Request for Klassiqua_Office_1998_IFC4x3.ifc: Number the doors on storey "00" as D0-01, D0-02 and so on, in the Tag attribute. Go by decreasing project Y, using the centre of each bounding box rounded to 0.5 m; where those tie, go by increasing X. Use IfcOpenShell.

First a look at what the model holds.

```python
import ifcopenshell
import ifcopenshell.util.element
import ifcopenshell.util.placement

model = ifcopenshell.open("Klassiqua_Office_1998_IFC4x3.ifc")
print(model.schema)
storey = next(s for s in model.by_type("IfcBuildingStorey") if s.Name == "00")
doors = [e for e in ifcopenshell.util.element.get_decomposition(storey) if e.is_a("IfcDoor")]
for e in sorted(doors, key=lambda e: e.id()):
    origin = ifcopenshell.util.placement.get_local_placement(e.ObjectPlacement)[:3, 3]
    print(e.id(), e.Tag, e.Name, origin.round(2) + 0.0, sep=" | ")
```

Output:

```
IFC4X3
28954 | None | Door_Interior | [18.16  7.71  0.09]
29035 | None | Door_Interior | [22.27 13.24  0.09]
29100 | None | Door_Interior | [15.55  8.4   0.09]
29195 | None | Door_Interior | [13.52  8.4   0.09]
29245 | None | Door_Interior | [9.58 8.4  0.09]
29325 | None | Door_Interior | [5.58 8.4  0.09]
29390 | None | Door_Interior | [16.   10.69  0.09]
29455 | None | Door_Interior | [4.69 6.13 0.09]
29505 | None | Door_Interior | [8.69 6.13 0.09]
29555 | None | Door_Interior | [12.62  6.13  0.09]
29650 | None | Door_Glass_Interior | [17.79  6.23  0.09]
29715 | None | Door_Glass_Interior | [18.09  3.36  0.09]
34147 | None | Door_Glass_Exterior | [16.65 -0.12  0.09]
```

```python
import ifcopenshell
import ifcopenshell.geom
import ifcopenshell.util.element
import ifcopenshell.util.shape

model = ifcopenshell.open("Klassiqua_Office_1998_IFC4x3.ifc")
settings = ifcopenshell.geom.settings()
settings.set("use-world-coords", True)


def centre(element):
    shape = ifcopenshell.geom.create_shape(settings, element)
    return ifcopenshell.util.shape.get_bbox_centroid(shape.geometry)


storey = next(s for s in model.by_type("IfcBuildingStorey") if s.Name == "00")
doors = [e for e in ifcopenshell.util.element.get_decomposition(storey) if e.is_a("IfcDoor")]

# Insertion points can sit at a corner or the storey origin, so sort by the geometry (in metres).
centres = {e: centre(e) for e in doors}
doors.sort(key=lambda e: (-round(centres[e][1] / 0.5), centres[e][0]))

for i, e in enumerate(doors, start=1):
    number = f"D0-{i:02d}"
    e.Tag = number
    print(e.id(), number)

model.write("Klassiqua_Office_1998_IFC4x3_rev.ifc")
```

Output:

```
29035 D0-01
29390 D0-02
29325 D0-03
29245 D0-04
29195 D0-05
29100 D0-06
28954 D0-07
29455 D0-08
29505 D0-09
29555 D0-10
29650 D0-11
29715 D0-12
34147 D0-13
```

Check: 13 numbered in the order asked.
